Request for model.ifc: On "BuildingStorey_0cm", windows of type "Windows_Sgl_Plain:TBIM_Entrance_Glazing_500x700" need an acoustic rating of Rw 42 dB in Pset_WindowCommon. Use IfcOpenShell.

First a look at what the model holds.

```python
import ifcopenshell
import ifcopenshell.util.element

model = ifcopenshell.open("model.ifc")
print(model.schema)
storey = next(s for s in model.by_type("IfcBuildingStorey") if s.Name == "BuildingStorey_0cm")
windows = [e for e in ifcopenshell.util.element.get_decomposition(storey) if e.is_a("IfcWindow")]
seen = {}
for e in windows:
    element_type = ifcopenshell.util.element.get_type(e)
    key = (element_type.Name if element_type != e and element_type else None, ifcopenshell.util.element.get_pset(e, "Pset_WindowCommon", "AcousticRating"))
    seen[key] = seen.get(key, 0) + 1
for (name, value), count in sorted(seen.items(), key=str):
    print(count, "x", name, "|", value)
```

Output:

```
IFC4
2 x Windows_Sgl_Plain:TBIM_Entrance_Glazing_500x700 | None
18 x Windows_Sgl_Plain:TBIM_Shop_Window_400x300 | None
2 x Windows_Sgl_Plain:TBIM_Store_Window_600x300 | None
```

```python
import ifcopenshell
import ifcopenshell.api.pset
import ifcopenshell.util.element

model = ifcopenshell.open("model.ifc")

storey = next(s for s in model.by_type("IfcBuildingStorey") if s.Name == "BuildingStorey_0cm")
windows = [e for e in ifcopenshell.util.element.get_decomposition(storey) if e.is_a("IfcWindow")]

count = 0
for e in windows:
    element_type = ifcopenshell.util.element.get_type(e)
    if element_type in (None, e) or element_type.Name != "Windows_Sgl_Plain:TBIM_Entrance_Glazing_500x700":
        continue
    # add_pset returns the element's existing set when there is one.
    pset = ifcopenshell.api.pset.add_pset(model, product=e, name="Pset_WindowCommon")
    ifcopenshell.api.pset.edit_pset(model, pset=pset, properties={"AcousticRating": "Rw 42 dB"})
    count += 1

print(count, "windows updated")

model.write("model_edited.ifc")
```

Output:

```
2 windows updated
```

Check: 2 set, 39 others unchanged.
